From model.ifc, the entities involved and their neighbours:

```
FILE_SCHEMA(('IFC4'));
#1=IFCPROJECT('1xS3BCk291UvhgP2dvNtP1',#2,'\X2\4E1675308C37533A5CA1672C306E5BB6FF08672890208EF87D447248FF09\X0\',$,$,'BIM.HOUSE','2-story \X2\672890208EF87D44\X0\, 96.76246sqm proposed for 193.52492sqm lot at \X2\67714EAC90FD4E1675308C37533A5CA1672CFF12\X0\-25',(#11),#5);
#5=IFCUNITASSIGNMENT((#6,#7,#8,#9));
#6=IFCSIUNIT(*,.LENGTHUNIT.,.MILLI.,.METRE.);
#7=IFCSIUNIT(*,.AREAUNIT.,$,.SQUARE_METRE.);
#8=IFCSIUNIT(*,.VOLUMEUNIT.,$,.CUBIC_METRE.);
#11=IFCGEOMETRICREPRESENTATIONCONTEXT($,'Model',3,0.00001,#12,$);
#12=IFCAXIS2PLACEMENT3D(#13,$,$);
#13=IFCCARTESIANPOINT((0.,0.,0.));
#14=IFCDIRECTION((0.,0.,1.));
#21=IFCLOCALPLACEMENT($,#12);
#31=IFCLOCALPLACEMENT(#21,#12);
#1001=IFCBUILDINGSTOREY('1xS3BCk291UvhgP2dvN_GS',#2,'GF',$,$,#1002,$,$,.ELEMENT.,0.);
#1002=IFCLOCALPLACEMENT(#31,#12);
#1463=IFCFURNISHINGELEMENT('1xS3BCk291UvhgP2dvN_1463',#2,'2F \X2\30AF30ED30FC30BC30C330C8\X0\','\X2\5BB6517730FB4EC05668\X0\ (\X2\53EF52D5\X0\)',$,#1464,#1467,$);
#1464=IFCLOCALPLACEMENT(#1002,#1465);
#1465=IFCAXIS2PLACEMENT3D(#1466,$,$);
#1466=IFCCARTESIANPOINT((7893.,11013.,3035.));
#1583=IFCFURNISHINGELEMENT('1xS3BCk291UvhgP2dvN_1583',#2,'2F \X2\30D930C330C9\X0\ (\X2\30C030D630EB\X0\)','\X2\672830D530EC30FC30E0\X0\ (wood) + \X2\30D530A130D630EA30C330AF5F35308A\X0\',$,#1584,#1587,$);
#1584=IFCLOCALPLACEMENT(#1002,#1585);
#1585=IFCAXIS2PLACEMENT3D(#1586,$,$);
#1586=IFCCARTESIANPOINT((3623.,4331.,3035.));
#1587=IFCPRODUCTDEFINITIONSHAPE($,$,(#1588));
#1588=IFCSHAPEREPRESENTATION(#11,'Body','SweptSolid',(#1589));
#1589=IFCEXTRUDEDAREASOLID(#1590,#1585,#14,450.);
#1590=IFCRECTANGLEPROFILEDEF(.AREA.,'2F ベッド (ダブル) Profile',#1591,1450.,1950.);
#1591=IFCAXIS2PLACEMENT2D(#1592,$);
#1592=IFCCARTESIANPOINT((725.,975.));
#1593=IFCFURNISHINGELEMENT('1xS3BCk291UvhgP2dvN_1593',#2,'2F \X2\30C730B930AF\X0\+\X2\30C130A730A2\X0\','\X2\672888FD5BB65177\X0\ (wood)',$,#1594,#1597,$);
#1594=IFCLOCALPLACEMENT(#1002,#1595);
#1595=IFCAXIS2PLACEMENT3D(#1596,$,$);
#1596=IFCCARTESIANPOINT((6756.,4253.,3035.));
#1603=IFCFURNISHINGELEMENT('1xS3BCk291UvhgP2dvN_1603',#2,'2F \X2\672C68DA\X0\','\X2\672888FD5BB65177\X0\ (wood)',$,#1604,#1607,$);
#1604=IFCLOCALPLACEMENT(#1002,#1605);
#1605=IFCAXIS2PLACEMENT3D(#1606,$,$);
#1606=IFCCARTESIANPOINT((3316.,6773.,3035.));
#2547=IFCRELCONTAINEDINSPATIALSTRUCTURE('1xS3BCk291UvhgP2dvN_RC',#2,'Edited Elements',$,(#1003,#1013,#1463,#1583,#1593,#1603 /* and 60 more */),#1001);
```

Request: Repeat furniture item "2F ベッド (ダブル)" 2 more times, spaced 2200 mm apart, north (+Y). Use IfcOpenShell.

```python
import numpy as np
import ifcopenshell
import ifcopenshell.api.geometry
import ifcopenshell.api.root
import ifcopenshell.util.element
import ifcopenshell.util.placement
import ifcopenshell.util.unit

model = ifcopenshell.open("model.ifc")
unit_scale = ifcopenshell.util.unit.calculate_unit_scale(model)


def reuse_history(source, copy):
    """copy_class also copies each property set's owner history, people and application; keep the originals."""
    for rel in copy.IsDefinedBy:
        if rel.is_a("IfcRelDefinesByProperties") and (history := rel.RelatingPropertyDefinition.OwnerHistory):
            rel.RelatingPropertyDefinition.OwnerHistory = source.OwnerHistory
            ifcopenshell.util.element.remove_deep2(model, history)


source = model.by_guid("1xS3BCk291UvhgP2dvN_1583")
base = ifcopenshell.util.placement.get_local_placement(source.ObjectPlacement)
step = np.array([0.0, 1.0, 0.0]) * 2.2 / unit_scale

for i in range(1, 3):
    copy = ifcopenshell.api.root.copy_class(model, product=source)
    copy.Representation = ifcopenshell.util.element.copy_deep(
        model, source.Representation, exclude=["IfcGeometricRepresentationContext", "IfcRepresentationMap"]
    )
    reuse_history(source, copy)
    matrix = base.copy()
    matrix[:3, 3] += i * step
    print("added at", matrix[:3, 3].round(3) + 0.0)
    ifcopenshell.api.geometry.edit_object_placement(model, product=copy, matrix=matrix, is_si=False)

model.write("model-out.ifc")
```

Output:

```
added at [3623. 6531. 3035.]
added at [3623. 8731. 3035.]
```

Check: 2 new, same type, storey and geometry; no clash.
